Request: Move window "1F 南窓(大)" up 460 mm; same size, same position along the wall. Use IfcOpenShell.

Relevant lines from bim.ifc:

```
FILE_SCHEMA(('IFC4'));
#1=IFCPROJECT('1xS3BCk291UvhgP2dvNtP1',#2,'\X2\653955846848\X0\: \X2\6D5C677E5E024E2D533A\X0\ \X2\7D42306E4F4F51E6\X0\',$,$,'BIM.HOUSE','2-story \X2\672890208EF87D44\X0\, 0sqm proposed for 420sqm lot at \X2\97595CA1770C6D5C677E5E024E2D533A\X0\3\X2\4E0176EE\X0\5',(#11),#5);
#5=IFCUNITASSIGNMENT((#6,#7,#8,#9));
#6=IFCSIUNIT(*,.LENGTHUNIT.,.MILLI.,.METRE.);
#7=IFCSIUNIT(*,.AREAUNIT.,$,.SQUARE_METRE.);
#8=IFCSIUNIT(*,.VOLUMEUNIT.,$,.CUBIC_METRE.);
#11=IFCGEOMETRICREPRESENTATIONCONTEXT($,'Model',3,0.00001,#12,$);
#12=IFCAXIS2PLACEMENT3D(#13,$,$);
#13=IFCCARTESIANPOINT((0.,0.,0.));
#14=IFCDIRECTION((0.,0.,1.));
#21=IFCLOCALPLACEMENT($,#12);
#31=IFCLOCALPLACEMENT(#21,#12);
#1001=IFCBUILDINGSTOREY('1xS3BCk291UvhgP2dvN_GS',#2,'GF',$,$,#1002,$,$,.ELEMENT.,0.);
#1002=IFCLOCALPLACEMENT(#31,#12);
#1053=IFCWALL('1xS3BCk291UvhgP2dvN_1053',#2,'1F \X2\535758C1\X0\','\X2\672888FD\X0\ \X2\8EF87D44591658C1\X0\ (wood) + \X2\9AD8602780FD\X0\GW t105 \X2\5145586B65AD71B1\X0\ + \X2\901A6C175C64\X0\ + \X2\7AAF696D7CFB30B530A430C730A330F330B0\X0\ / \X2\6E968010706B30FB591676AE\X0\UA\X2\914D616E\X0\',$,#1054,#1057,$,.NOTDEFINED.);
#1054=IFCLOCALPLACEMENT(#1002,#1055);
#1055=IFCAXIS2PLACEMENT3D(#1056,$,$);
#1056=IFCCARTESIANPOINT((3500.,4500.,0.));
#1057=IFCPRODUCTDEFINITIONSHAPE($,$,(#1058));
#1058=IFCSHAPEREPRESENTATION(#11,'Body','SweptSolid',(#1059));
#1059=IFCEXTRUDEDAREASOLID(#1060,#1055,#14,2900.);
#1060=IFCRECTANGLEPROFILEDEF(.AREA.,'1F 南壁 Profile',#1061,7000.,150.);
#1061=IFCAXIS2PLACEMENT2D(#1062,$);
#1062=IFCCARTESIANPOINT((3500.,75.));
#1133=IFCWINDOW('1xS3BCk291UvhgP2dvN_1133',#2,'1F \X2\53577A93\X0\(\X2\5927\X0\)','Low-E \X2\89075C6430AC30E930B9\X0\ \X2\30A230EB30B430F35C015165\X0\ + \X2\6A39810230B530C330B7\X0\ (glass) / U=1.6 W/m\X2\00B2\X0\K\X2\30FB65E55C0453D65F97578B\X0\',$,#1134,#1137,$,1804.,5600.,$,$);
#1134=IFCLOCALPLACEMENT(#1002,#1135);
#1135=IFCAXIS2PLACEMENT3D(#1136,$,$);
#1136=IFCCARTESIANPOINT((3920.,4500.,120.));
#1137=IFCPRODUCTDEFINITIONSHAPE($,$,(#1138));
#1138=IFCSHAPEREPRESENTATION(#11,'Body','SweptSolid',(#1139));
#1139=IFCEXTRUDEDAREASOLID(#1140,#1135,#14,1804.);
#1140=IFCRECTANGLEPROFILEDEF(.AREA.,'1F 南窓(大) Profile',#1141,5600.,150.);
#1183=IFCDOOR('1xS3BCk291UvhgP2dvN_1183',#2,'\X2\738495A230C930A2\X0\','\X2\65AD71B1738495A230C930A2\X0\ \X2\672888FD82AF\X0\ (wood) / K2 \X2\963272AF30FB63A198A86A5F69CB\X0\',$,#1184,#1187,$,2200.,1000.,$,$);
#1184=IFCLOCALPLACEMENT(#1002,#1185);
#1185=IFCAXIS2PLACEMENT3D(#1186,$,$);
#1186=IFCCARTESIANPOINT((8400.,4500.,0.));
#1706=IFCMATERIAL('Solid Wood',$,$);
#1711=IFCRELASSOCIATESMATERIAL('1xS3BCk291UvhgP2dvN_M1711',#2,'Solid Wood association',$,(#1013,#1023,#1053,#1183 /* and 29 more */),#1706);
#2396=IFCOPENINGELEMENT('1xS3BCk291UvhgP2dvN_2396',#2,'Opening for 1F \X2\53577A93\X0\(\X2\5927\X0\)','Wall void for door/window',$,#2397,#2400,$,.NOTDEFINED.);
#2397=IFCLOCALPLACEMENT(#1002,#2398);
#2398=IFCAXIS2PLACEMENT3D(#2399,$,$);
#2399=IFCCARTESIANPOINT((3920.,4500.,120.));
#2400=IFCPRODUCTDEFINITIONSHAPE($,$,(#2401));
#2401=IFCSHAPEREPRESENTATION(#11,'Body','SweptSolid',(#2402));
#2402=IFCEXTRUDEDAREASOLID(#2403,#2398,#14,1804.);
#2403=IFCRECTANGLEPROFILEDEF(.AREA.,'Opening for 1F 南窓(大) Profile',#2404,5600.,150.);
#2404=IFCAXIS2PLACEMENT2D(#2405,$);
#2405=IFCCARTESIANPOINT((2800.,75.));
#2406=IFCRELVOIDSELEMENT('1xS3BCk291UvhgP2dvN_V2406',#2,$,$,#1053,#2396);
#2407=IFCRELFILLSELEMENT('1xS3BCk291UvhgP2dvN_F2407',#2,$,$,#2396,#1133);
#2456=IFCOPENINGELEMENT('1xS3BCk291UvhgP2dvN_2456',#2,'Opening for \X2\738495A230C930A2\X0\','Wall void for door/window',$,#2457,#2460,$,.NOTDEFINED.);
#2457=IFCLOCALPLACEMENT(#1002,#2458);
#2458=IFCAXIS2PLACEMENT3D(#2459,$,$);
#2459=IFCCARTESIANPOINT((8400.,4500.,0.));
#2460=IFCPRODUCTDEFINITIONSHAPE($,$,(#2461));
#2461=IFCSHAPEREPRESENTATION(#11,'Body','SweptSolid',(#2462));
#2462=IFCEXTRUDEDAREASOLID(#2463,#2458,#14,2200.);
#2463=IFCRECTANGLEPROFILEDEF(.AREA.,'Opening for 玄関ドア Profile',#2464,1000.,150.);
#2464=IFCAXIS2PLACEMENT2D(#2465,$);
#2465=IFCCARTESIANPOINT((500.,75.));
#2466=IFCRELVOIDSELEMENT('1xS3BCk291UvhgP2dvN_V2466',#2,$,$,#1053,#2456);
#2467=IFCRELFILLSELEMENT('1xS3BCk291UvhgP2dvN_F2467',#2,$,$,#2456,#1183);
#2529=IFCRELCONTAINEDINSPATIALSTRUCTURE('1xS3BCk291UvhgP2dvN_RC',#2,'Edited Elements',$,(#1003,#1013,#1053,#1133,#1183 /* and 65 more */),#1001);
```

```python
import numpy as np
import ifcopenshell
import ifcopenshell.api.geometry
import ifcopenshell.util.placement
import ifcopenshell.util.unit

model = ifcopenshell.open("bim.ifc")
unit_scale = ifcopenshell.util.unit.calculate_unit_scale(model)

window = model.by_id(1133)
opening = window.FillsVoids[0].RelatingOpeningElement
dz = 0.46 / unit_scale

shift = np.array([0.0, 0.0, dz])
# The window is not placed relative to its opening, so move both.
for product in (opening, window):
    matrix = ifcopenshell.util.placement.get_local_placement(product.ObjectPlacement)
    matrix[:3, 3] += shift
    ifcopenshell.api.geometry.edit_object_placement(model, product=product, matrix=matrix, is_si=False)

print(f"moved by {dz * unit_scale:+.3f} m")

model.write("bim_edited.ifc")
```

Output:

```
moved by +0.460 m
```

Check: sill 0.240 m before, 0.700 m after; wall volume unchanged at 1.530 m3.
